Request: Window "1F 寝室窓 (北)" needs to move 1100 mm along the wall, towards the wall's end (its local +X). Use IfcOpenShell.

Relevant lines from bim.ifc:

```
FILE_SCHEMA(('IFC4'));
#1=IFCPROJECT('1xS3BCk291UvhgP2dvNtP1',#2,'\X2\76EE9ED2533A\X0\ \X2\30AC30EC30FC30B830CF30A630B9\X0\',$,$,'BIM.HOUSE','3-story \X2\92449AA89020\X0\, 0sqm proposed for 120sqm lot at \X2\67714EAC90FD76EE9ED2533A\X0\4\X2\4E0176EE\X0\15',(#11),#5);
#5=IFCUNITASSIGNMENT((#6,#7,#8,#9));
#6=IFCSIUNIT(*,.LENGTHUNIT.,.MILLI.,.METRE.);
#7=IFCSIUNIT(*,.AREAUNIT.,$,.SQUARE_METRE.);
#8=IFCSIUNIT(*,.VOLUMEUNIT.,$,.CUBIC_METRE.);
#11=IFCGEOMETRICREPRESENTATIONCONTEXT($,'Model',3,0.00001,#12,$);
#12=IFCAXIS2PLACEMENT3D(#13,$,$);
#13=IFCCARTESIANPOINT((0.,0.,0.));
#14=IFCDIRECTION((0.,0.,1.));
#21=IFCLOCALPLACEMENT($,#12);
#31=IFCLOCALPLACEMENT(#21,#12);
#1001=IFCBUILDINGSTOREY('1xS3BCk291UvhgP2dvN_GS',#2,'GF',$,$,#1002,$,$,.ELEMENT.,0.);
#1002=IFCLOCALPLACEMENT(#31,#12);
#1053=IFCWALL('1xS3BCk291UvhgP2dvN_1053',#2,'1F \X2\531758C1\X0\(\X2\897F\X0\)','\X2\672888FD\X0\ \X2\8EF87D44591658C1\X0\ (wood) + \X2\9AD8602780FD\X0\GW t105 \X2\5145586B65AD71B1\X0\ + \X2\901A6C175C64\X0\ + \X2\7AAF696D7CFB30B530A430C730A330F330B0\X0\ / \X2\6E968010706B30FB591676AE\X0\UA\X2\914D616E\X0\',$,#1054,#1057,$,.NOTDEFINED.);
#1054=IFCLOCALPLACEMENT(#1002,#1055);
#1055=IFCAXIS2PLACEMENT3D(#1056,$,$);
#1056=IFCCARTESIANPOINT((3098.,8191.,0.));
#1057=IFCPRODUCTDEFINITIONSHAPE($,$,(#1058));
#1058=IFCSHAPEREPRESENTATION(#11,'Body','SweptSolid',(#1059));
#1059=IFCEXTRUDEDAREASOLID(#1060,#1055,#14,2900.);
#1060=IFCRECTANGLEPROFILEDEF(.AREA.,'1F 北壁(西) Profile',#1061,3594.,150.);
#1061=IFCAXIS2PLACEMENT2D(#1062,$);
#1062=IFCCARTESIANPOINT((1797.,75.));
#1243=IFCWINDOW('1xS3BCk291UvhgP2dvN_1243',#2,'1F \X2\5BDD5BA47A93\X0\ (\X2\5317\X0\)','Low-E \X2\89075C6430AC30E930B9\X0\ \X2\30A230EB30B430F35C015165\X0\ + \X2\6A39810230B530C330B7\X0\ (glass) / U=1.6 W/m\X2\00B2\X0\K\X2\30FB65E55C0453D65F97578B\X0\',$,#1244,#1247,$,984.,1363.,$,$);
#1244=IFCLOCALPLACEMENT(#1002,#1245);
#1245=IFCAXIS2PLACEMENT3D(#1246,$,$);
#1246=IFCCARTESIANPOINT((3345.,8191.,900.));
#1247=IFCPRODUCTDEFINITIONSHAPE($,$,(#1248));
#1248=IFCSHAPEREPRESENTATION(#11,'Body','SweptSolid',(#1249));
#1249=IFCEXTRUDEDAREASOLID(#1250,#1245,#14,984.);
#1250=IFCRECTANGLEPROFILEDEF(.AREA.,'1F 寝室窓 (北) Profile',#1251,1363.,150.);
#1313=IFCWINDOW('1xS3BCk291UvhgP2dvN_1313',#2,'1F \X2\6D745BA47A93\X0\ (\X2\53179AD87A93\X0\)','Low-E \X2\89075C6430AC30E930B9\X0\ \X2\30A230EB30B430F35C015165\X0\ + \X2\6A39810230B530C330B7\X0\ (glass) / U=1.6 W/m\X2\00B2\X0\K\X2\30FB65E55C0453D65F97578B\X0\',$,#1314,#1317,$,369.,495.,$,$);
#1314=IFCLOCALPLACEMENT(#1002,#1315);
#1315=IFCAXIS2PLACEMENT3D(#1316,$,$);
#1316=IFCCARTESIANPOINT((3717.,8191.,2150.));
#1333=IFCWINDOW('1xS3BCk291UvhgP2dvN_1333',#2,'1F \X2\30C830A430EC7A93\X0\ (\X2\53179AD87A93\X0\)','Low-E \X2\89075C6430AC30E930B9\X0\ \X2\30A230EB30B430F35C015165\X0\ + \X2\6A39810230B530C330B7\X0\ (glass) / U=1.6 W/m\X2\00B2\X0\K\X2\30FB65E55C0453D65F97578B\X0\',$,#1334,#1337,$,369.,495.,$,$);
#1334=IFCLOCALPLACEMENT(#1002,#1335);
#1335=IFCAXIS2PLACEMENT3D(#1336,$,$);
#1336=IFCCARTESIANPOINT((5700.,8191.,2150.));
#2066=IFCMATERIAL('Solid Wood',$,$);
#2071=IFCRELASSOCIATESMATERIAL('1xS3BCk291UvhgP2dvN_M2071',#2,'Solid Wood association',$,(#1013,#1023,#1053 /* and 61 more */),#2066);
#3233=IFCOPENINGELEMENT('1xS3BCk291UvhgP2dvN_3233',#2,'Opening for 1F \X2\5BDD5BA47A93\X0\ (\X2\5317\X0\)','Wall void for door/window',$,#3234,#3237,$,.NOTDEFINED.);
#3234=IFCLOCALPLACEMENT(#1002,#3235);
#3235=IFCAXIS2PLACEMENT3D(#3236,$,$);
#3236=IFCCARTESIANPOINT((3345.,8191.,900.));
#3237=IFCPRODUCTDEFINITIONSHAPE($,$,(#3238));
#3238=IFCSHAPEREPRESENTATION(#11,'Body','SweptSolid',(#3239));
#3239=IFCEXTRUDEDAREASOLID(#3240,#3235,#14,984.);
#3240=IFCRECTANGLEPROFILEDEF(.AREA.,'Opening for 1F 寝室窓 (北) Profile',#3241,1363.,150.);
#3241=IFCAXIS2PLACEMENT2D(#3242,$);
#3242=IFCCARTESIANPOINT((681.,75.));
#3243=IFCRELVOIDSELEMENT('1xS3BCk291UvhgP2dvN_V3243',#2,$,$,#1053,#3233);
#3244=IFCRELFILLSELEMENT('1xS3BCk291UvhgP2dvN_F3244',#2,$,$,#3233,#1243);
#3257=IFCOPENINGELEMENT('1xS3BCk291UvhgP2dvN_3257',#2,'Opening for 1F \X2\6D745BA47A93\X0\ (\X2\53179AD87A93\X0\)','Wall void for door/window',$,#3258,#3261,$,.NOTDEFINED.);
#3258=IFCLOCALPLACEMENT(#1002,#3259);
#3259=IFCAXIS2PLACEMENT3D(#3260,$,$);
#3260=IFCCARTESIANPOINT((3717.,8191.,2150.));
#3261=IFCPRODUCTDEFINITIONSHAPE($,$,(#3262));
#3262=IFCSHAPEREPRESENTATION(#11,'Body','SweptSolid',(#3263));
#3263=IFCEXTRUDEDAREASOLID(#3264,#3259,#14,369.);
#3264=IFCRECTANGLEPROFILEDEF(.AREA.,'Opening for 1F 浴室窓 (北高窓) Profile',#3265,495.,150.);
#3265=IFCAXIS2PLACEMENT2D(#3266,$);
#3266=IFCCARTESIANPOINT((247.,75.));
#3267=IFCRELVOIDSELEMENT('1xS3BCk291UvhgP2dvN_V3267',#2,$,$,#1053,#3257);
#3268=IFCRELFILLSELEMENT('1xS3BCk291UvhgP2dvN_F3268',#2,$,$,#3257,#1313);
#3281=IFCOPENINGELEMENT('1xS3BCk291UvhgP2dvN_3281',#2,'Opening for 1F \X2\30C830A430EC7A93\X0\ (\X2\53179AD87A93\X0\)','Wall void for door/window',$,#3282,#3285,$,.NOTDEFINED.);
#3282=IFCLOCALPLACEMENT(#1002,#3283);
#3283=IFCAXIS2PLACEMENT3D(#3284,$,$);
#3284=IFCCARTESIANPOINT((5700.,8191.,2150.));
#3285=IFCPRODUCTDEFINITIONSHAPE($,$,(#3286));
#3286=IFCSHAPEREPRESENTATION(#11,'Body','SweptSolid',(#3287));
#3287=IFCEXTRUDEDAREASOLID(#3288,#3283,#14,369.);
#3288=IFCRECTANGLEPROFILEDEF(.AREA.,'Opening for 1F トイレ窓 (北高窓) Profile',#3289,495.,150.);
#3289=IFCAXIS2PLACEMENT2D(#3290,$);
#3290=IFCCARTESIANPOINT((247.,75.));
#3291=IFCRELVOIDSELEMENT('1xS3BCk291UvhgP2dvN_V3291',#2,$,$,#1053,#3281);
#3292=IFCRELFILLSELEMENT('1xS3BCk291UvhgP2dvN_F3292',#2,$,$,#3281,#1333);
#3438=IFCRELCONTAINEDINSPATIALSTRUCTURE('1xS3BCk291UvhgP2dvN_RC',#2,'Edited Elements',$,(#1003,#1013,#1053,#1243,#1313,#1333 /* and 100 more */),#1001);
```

```python
import ifcopenshell
import ifcopenshell.api.geometry
import ifcopenshell.util.placement

model = ifcopenshell.open("bim.ifc")

window = model.by_guid("1xS3BCk291UvhgP2dvN_1243")
opening = window.FillsVoids[0].RelatingOpeningElement
wall = opening.VoidsElements[0].RelatingBuildingElement

wall_matrix = ifcopenshell.util.placement.get_local_placement(wall.ObjectPlacement)
shift = wall_matrix[:3, 0] * 1100.0
before = ifcopenshell.util.placement.get_local_placement(window.ObjectPlacement)[:3, 3].copy()

# The window is not placed relative to its opening, so move both.
for product in (opening, window):
    matrix = ifcopenshell.util.placement.get_local_placement(product.ObjectPlacement)
    matrix[:3, 3] += shift
    ifcopenshell.api.geometry.edit_object_placement(model, product=product, matrix=matrix, is_si=False)

after = ifcopenshell.util.placement.get_local_placement(window.ObjectPlacement)[:3, 3]
print("window moved by", (after - before).round(3) + 0.0)

model.write("bim_edited.ifc")
```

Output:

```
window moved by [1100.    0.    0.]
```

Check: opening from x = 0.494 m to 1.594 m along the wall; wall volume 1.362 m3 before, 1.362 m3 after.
